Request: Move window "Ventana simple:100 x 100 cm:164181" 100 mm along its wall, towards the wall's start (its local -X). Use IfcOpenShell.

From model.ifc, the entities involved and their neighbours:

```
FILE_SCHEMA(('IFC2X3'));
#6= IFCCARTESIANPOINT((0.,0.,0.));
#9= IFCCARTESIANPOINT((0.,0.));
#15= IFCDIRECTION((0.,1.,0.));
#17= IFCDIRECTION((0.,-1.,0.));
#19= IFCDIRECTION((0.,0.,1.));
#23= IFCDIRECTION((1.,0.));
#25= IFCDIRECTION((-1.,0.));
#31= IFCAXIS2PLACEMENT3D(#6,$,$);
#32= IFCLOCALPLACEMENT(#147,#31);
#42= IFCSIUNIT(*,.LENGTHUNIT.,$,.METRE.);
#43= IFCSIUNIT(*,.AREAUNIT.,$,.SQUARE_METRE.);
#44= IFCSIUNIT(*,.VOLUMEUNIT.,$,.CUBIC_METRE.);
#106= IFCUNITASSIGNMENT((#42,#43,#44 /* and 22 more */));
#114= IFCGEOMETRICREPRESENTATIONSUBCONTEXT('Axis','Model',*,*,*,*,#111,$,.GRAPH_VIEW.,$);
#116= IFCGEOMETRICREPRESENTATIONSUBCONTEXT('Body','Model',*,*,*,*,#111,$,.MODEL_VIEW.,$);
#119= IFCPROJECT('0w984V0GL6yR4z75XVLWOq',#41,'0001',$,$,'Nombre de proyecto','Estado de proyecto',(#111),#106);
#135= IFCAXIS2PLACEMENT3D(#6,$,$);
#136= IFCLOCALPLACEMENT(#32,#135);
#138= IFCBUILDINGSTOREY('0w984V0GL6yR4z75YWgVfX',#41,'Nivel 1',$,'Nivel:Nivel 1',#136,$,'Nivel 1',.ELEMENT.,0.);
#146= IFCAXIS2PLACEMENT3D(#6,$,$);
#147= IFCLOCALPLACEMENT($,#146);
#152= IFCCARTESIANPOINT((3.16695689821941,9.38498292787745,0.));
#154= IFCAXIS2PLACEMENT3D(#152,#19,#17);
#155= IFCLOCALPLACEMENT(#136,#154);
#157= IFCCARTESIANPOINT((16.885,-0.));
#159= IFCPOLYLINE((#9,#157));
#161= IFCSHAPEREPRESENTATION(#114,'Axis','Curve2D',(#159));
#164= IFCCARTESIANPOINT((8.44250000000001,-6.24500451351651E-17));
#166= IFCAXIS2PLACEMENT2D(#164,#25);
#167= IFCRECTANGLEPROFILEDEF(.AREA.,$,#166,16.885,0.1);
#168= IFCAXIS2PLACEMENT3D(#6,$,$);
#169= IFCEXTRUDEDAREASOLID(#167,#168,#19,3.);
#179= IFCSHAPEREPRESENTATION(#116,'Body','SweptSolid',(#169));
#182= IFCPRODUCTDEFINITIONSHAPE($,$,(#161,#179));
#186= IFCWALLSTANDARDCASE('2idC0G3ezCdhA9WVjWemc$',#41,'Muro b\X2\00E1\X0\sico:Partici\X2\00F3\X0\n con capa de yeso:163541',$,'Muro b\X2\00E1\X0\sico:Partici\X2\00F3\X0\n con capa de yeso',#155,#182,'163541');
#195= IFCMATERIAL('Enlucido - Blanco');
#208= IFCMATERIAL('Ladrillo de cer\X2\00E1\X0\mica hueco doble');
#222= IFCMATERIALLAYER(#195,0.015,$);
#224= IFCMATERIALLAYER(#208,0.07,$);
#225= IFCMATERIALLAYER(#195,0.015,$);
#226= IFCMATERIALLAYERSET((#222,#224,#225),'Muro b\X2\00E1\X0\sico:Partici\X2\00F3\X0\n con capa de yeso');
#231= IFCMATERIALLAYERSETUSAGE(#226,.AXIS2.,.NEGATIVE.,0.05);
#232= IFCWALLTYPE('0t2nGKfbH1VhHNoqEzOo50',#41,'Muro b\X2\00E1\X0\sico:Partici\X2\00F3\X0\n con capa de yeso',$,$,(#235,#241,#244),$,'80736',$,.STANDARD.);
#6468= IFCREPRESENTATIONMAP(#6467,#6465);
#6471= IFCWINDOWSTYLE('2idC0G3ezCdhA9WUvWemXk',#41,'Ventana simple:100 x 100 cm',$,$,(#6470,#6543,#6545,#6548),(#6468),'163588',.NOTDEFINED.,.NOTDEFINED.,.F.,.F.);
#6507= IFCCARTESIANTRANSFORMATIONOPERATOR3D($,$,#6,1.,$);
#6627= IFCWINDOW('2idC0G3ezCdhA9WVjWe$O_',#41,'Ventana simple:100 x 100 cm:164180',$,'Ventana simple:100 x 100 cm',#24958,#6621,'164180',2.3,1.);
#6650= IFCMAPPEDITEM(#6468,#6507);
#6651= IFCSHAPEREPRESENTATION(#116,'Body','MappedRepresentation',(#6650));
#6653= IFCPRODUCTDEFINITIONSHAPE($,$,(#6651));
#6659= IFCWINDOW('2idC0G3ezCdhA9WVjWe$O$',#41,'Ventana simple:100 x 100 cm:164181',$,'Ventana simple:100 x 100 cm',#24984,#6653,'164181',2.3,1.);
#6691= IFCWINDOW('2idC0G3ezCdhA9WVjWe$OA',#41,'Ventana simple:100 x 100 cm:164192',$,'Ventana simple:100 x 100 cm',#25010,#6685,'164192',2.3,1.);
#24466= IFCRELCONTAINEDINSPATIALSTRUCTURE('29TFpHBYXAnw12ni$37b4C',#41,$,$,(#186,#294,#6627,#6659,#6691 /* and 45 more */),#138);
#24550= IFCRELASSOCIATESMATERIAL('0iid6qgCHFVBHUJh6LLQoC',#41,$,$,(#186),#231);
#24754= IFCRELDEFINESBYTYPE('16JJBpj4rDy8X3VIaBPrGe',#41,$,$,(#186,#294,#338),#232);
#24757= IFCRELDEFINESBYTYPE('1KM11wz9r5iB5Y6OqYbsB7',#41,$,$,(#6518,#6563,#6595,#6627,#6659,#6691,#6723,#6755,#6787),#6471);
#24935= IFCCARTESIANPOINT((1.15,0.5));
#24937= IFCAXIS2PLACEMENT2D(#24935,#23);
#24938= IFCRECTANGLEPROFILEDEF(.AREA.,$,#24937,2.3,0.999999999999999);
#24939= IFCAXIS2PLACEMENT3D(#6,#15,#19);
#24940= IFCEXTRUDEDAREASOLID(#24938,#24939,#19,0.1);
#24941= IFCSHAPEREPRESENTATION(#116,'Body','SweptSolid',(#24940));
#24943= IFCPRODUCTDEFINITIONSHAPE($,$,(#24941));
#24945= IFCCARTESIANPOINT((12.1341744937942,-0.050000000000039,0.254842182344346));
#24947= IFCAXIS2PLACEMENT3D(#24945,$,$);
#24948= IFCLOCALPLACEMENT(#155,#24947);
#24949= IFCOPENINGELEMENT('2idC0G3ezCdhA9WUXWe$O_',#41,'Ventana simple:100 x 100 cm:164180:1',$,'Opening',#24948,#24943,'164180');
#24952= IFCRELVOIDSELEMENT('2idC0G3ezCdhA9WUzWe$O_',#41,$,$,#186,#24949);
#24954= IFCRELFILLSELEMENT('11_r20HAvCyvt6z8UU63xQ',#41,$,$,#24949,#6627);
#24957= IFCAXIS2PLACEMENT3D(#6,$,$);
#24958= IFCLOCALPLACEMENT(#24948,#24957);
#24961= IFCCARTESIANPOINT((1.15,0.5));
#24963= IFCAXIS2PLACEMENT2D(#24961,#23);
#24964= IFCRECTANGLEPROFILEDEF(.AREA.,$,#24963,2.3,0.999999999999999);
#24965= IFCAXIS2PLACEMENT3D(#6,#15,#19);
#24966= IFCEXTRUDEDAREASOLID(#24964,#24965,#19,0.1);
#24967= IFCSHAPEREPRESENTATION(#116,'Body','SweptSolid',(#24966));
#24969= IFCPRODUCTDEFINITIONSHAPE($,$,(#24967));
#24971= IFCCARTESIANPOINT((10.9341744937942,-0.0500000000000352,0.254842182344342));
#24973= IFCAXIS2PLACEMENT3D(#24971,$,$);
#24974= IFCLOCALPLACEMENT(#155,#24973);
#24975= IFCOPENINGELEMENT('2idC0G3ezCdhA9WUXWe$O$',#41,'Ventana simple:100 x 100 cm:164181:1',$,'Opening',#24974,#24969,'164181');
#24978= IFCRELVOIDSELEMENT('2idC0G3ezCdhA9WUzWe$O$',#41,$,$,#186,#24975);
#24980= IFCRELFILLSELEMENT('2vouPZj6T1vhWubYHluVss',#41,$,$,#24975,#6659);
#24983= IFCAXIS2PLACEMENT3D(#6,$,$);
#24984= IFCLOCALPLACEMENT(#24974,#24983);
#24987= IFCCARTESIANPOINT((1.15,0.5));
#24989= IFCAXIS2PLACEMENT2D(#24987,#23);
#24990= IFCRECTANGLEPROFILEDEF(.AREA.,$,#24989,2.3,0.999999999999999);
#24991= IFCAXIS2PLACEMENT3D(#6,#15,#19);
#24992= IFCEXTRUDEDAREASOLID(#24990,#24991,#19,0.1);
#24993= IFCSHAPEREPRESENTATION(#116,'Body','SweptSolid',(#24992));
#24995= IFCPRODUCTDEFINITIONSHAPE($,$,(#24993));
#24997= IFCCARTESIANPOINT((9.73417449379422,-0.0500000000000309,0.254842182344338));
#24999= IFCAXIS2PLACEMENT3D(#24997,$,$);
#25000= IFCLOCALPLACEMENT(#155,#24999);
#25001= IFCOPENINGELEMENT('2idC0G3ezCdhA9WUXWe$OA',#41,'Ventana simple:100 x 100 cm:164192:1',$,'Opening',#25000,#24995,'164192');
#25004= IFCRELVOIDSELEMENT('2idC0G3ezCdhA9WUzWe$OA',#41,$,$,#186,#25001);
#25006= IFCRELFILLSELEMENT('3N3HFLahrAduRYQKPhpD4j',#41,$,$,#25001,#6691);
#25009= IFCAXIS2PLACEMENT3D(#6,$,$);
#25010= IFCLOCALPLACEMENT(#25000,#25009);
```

```python
import ifcopenshell
import ifcopenshell.api.geometry
import ifcopenshell.util.placement
import ifcopenshell.util.unit

model = ifcopenshell.open("model.ifc")
unit_scale = ifcopenshell.util.unit.calculate_unit_scale(model)

window = model.by_guid("2idC0G3ezCdhA9WVjWe$O$")
opening = window.FillsVoids[0].RelatingOpeningElement
wall = opening.VoidsElements[0].RelatingBuildingElement

wall_matrix = ifcopenshell.util.placement.get_local_placement(wall.ObjectPlacement)
shift = wall_matrix[:3, 0] * -0.1 / unit_scale
before = ifcopenshell.util.placement.get_local_placement(window.ObjectPlacement)[:3, 3].copy()

# The window is placed relative to its opening, so it follows when the opening moves.
matrix = ifcopenshell.util.placement.get_local_placement(opening.ObjectPlacement)
matrix[:3, 3] += shift
ifcopenshell.api.geometry.edit_object_placement(
    model, product=opening, matrix=matrix, is_si=False, should_transform_children=True
)

after = ifcopenshell.util.placement.get_local_placement(window.ObjectPlacement)[:3, 3]
print("window moved by", (after - before).round(3) + 0.0)

model.write("model_updated.ifc")
```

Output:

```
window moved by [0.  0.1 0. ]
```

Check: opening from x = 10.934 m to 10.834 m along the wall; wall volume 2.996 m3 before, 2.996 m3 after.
